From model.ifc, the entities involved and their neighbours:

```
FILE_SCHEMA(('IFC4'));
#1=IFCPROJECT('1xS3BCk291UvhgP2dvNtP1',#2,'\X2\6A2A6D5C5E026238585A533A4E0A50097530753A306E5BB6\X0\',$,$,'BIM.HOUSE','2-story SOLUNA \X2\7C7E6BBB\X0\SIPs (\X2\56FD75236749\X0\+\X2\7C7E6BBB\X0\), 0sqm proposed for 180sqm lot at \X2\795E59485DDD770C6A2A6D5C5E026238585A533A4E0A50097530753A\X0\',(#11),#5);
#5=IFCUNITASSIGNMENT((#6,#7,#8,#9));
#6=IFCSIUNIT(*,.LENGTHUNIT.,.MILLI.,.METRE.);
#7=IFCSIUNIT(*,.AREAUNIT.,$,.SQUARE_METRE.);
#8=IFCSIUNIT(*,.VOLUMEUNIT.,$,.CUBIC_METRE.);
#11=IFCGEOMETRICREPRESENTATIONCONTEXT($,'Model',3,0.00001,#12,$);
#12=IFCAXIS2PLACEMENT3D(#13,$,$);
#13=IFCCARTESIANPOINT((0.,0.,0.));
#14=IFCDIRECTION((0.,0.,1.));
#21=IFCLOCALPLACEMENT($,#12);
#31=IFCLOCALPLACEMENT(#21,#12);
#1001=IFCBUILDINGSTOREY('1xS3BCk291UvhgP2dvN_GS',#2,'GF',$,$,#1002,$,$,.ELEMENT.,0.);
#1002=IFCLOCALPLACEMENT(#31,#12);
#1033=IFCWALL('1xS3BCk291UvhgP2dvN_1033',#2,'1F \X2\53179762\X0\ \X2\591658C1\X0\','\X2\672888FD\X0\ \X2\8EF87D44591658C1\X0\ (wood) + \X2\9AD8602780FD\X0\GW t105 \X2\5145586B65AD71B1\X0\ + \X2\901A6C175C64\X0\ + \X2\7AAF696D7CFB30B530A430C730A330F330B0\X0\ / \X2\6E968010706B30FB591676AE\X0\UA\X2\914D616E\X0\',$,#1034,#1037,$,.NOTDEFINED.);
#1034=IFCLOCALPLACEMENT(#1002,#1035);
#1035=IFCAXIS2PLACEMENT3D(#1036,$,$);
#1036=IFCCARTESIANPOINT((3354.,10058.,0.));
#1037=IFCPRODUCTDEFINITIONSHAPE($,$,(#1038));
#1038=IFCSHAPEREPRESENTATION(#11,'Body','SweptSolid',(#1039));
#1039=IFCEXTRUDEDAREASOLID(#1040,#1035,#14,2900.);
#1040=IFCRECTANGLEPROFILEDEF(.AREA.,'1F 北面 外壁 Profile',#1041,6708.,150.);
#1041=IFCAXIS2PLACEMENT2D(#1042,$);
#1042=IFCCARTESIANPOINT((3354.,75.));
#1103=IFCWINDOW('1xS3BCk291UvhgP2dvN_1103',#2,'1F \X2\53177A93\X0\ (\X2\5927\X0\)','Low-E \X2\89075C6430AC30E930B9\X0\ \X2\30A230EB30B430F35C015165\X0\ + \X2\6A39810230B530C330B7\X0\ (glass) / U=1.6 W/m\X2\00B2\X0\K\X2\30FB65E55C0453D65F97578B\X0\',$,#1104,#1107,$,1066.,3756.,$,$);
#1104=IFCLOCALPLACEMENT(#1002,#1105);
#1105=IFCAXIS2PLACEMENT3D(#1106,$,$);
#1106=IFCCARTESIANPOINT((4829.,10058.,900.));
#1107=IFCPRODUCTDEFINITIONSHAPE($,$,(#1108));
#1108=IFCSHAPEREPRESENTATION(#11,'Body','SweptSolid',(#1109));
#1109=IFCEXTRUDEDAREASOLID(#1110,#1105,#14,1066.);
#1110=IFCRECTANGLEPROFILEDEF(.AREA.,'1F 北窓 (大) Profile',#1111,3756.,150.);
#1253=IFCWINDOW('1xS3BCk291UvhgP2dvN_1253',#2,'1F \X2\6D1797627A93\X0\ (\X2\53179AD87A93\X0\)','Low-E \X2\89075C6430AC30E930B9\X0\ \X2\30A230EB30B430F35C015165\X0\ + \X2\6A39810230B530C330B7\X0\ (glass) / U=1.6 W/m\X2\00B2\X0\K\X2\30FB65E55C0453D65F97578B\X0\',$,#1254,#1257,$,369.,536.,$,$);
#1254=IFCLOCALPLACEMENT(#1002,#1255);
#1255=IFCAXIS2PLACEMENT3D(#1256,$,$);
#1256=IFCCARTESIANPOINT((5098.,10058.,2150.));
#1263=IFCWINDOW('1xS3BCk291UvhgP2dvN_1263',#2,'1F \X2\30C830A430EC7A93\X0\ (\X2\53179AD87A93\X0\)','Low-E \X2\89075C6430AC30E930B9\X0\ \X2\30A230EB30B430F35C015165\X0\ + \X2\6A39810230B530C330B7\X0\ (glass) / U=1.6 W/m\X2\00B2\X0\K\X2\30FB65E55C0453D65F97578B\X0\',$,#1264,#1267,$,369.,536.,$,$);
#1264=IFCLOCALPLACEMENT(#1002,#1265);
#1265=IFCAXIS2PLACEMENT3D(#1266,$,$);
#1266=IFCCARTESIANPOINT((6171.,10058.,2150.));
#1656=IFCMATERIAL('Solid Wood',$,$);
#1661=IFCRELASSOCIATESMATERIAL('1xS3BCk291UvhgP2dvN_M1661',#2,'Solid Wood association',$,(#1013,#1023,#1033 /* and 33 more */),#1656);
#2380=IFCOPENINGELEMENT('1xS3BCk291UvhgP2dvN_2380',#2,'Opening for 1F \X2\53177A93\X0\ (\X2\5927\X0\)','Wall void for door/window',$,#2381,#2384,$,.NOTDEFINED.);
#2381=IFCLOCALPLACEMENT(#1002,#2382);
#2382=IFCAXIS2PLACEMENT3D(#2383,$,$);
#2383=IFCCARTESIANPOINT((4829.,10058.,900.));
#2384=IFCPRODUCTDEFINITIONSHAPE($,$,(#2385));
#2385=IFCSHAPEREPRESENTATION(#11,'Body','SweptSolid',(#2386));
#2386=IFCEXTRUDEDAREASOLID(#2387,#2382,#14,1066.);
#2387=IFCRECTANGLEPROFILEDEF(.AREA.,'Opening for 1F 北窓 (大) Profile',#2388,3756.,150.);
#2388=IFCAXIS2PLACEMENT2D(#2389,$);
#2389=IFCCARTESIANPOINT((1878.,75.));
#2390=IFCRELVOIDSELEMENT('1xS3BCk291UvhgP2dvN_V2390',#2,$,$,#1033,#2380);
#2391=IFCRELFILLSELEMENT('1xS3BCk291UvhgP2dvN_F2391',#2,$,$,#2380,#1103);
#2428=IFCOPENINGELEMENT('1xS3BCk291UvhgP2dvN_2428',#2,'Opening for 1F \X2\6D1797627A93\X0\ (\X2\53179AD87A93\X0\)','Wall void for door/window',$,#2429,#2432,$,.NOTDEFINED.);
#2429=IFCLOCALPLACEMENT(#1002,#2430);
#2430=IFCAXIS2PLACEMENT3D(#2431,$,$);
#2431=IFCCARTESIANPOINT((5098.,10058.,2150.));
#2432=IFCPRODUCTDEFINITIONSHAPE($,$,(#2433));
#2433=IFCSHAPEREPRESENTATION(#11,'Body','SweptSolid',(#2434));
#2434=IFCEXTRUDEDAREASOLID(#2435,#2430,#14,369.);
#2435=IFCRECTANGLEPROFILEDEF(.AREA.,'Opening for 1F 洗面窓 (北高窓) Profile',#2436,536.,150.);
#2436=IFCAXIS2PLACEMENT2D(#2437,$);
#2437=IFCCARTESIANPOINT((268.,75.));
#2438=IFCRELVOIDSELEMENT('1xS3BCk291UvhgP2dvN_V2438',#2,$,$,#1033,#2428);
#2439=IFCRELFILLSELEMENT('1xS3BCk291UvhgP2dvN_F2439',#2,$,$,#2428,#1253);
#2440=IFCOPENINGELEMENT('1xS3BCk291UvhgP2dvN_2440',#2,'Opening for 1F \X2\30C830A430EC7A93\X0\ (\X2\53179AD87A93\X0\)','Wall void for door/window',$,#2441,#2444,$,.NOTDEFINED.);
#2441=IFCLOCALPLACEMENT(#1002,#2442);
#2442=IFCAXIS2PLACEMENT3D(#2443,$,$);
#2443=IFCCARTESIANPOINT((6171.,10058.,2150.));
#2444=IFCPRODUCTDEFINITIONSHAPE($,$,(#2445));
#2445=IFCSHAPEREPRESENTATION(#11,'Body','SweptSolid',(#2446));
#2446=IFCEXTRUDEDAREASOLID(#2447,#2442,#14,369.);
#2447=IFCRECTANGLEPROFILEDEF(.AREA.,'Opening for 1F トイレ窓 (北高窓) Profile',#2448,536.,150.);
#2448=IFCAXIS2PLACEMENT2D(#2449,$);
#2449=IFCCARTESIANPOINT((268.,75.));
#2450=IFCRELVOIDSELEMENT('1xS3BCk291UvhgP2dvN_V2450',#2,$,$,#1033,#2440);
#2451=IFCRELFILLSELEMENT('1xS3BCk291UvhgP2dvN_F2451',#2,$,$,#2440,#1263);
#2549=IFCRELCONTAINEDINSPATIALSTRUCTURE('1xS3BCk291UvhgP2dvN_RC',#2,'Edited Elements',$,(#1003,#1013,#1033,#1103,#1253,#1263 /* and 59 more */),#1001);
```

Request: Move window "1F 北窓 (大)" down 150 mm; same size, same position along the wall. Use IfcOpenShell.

```python
import numpy as np
import ifcopenshell
import ifcopenshell.api.geometry
import ifcopenshell.util.placement
import ifcopenshell.util.unit

model = ifcopenshell.open("model.ifc")
unit_scale = ifcopenshell.util.unit.calculate_unit_scale(model)

window = model.by_id(1103)
opening = window.FillsVoids[0].RelatingOpeningElement
dz = -150.0

shift = np.array([0.0, 0.0, dz])
# The window is not placed relative to its opening, so move both.
for product in (opening, window):
    matrix = ifcopenshell.util.placement.get_local_placement(product.ObjectPlacement)
    matrix[:3, 3] += shift
    ifcopenshell.api.geometry.edit_object_placement(model, product=product, matrix=matrix, is_si=False)

print(f"moved by {dz * unit_scale:+.3f} m")

model.write("model_edited.ifc")
```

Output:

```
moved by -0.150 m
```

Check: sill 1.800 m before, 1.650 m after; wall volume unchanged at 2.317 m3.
